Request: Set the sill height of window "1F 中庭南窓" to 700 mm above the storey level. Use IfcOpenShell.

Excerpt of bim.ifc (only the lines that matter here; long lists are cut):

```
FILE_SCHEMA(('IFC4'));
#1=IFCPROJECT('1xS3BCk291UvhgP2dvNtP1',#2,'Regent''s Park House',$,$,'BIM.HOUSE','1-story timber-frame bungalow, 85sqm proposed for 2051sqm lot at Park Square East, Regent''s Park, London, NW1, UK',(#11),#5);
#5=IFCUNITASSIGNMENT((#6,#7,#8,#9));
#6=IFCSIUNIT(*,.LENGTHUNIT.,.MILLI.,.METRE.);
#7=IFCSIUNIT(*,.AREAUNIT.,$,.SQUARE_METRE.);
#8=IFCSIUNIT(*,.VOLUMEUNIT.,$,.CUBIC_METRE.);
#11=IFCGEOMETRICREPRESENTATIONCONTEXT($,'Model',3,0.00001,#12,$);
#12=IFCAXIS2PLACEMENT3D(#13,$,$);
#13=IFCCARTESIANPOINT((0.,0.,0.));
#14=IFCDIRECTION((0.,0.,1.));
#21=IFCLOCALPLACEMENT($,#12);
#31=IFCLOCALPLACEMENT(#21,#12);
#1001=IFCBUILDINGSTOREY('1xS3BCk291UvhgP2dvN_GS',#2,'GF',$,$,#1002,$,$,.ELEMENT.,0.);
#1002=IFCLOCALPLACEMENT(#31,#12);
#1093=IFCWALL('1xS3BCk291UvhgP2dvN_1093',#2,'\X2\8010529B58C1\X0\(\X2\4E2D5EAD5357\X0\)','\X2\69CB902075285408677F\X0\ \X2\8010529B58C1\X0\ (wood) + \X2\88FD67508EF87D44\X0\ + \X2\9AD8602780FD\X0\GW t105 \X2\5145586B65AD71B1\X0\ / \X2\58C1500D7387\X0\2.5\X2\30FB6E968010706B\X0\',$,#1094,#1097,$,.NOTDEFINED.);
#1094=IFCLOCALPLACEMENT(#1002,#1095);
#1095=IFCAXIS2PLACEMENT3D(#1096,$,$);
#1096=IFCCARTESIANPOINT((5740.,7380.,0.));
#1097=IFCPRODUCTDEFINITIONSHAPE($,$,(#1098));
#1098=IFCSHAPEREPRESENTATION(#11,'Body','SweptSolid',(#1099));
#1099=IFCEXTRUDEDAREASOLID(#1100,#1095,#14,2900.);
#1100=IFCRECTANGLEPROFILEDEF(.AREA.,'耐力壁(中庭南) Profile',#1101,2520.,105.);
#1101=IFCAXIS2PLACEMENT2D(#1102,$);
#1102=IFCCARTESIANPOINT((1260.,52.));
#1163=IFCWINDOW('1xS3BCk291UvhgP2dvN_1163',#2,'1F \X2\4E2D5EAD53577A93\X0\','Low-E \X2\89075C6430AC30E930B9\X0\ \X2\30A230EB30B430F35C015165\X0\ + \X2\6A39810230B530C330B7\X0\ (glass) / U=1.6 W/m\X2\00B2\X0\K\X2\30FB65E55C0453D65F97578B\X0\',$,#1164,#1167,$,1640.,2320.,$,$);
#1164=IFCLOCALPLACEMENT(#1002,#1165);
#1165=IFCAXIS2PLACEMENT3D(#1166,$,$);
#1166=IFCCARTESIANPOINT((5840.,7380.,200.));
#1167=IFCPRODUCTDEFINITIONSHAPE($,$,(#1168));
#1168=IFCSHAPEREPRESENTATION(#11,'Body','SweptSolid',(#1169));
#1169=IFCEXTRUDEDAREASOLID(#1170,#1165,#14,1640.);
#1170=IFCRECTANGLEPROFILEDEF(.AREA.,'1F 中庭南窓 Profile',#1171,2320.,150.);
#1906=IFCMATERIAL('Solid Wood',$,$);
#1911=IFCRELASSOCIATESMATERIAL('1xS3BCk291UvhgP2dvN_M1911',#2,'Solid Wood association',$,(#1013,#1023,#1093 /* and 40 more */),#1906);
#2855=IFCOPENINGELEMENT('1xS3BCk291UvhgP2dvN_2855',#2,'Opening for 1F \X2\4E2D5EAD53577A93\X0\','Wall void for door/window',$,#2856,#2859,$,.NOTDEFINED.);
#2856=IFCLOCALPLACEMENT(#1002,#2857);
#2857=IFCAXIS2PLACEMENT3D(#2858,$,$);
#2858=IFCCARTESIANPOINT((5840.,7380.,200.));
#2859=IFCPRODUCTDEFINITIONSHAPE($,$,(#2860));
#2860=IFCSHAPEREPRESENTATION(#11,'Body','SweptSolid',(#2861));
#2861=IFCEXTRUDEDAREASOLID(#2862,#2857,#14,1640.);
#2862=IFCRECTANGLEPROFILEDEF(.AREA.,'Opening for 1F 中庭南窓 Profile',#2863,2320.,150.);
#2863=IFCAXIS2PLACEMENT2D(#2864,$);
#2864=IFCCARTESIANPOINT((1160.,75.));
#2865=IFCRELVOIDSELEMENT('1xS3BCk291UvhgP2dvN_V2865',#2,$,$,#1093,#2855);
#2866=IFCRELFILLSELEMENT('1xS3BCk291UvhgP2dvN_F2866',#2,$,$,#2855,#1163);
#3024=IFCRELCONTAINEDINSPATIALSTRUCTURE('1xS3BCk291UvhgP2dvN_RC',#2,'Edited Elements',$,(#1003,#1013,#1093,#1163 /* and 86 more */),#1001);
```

```python
import numpy as np
import ifcopenshell
import ifcopenshell.api.geometry
import ifcopenshell.geom
import ifcopenshell.util.element
import ifcopenshell.util.placement
import ifcopenshell.util.shape
import ifcopenshell.util.unit

model = ifcopenshell.open("bim.ifc")
unit_scale = ifcopenshell.util.unit.calculate_unit_scale(model)

window = model.by_guid("1xS3BCk291UvhgP2dvN_1163")
opening = window.FillsVoids[0].RelatingOpeningElement
storey = ifcopenshell.util.element.get_container(window, ifc_class="IfcBuildingStorey")
level = ifcopenshell.util.placement.get_local_placement(storey.ObjectPlacement)[2, 3]

# The opening's origin need not be at the sill, so measure its lowest point.
shape = ifcopenshell.geom.create_shape(ifcopenshell.geom.settings(), opening)
bottom = ifcopenshell.util.shape.get_shape_bottom_elevation(shape, shape.geometry) / unit_scale
dz = level + 700.0 - bottom

shift = np.array([0.0, 0.0, dz])
# The window is not placed relative to its opening, so move both.
for product in (opening, window):
    matrix = ifcopenshell.util.placement.get_local_placement(product.ObjectPlacement)
    matrix[:3, 3] += shift
    ifcopenshell.api.geometry.edit_object_placement(model, product=product, matrix=matrix, is_si=False)

print(f"moved by {dz * unit_scale:+.3f} m")

model.write("bim_edited.ifc")
```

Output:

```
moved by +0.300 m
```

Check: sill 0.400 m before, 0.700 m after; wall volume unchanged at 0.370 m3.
